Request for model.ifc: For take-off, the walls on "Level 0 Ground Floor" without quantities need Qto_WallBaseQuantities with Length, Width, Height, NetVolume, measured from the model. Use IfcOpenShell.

First a look at what the model holds.

```python
import ifcopenshell
import ifcopenshell.util.element
import ifcopenshell.util.unit

model = ifcopenshell.open("model.ifc")
print(model.schema)
for unit_type in ("LENGTHUNIT", "AREAUNIT", "VOLUMEUNIT"):
    print(unit_type, ifcopenshell.util.unit.calculate_unit_scale(model, unit_type))
storey = next(s for s in model.by_type("IfcBuildingStorey") if s.Name == "Level 0 Ground Floor")
walls = [e for e in ifcopenshell.util.element.get_decomposition(storey) if e.is_a("IfcWall")]
for e in sorted(walls, key=lambda e: e.id()):
    print(e.id(), e.is_a(), e.Name, list(ifcopenshell.util.element.get_psets(e, qtos_only=True)), sep=" | ")
```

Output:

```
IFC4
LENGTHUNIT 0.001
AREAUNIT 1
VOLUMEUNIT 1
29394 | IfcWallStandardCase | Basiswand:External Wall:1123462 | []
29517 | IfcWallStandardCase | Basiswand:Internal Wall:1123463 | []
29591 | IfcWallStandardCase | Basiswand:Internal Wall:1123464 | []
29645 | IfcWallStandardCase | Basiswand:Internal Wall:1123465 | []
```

```python
import ifcopenshell
import ifcopenshell.api.pset
import ifcopenshell.geom
import ifcopenshell.util.element
import ifcopenshell.util.shape
import ifcopenshell.util.unit

model = ifcopenshell.open("model.ifc")
unit_scale = ifcopenshell.util.unit.calculate_unit_scale(model)
volume_scale = ifcopenshell.util.unit.calculate_unit_scale(model, "VOLUMEUNIT")
settings = ifcopenshell.geom.settings()

storey = next(s for s in model.by_type("IfcBuildingStorey") if s.Name == "Level 0 Ground Floor")
walls = [e for e in ifcopenshell.util.element.get_decomposition(storey) if e.is_a("IfcWall")]

for e in sorted(walls, key=lambda e: e.id()):
    if ifcopenshell.util.element.get_psets(e, qtos_only=True, should_inherit=False):
        continue
    # Geometry comes back in metres, in the element's own axes.
    shape = ifcopenshell.geom.create_shape(settings, e)
    values = {
        "Length": ifcopenshell.util.shape.get_x(shape.geometry) / unit_scale,
        "Width": ifcopenshell.util.shape.get_y(shape.geometry) / unit_scale,
        "Height": ifcopenshell.util.shape.get_z(shape.geometry) / unit_scale,
        "NetVolume": ifcopenshell.util.shape.get_volume(shape.geometry) / volume_scale,
    }
    qto = ifcopenshell.api.pset.add_qto(model, product=e, name="Qto_WallBaseQuantities")
    ifcopenshell.api.pset.edit_qto(model, qto=qto, properties=values)
    print(e.id(), {k: round(v, 3) for k, v in values.items()})

model.write("model_rev.ifc")
```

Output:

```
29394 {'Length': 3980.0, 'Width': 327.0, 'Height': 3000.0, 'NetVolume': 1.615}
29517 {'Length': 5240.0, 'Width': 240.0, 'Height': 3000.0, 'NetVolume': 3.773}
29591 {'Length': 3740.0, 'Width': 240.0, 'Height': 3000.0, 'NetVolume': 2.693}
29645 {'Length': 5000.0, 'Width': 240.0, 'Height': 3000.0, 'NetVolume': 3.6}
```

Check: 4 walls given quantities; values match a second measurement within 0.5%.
